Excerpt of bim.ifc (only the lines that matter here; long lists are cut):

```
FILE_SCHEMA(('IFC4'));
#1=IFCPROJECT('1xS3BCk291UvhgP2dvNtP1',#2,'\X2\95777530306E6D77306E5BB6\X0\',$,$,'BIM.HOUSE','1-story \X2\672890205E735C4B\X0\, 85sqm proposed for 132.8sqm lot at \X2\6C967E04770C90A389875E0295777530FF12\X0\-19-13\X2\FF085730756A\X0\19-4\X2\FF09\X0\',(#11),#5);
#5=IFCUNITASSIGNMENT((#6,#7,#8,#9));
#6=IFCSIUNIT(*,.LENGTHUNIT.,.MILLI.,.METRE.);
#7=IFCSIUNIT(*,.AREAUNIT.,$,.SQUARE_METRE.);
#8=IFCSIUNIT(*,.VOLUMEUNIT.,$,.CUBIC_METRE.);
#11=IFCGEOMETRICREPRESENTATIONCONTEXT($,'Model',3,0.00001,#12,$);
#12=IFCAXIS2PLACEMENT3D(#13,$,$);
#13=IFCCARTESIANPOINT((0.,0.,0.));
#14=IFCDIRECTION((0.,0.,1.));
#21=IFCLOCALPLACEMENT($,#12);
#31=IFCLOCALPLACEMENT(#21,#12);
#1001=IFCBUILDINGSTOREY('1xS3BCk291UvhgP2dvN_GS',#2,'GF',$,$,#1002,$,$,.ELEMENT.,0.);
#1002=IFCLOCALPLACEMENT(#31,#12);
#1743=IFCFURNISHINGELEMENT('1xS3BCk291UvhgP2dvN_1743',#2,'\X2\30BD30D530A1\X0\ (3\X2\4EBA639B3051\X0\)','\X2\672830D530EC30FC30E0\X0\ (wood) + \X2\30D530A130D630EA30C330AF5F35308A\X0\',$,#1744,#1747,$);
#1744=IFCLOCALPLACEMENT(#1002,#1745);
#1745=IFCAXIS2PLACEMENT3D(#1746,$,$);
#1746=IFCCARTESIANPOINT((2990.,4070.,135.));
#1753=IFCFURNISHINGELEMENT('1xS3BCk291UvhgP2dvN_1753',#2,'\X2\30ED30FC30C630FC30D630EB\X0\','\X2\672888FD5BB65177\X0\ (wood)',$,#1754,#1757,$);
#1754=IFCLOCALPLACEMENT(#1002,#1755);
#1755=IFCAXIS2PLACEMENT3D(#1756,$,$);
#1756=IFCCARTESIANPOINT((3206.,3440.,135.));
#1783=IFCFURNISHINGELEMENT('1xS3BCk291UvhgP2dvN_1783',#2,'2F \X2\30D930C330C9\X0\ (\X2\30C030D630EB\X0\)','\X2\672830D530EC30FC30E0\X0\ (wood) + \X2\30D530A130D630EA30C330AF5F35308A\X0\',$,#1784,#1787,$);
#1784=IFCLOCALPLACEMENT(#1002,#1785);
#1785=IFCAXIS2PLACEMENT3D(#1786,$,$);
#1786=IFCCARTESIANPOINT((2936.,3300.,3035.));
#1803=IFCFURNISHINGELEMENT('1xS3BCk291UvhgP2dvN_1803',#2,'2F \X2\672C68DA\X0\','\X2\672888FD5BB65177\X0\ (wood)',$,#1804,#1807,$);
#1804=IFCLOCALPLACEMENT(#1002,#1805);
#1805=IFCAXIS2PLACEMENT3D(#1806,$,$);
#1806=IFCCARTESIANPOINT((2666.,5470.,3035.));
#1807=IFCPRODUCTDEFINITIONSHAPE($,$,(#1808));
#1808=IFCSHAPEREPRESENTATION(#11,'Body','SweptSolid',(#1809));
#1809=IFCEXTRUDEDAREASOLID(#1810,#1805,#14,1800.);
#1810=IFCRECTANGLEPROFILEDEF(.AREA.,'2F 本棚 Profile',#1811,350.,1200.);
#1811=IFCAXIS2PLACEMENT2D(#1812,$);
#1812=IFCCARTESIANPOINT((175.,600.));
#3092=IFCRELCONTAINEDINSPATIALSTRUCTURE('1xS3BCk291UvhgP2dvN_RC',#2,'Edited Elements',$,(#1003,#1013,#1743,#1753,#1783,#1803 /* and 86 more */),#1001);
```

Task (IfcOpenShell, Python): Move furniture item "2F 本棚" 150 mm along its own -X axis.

```python
import ifcopenshell
import ifcopenshell.api.geometry
import ifcopenshell.util.placement
import ifcopenshell.util.unit

model = ifcopenshell.open("bim.ifc")
unit_scale = ifcopenshell.util.unit.calculate_unit_scale(model)

item = model.by_guid("1xS3BCk291UvhgP2dvN_1803")
matrix = ifcopenshell.util.placement.get_local_placement(item.ObjectPlacement)
matrix[:3, 3] -= matrix[:3, 0] * 0.15 / unit_scale
ifcopenshell.api.geometry.edit_object_placement(model, product=item, matrix=matrix, is_si=False)

print(ifcopenshell.util.placement.get_local_placement(item.ObjectPlacement).round(3) + 0.0)

model.write("bim_v2.ifc")
```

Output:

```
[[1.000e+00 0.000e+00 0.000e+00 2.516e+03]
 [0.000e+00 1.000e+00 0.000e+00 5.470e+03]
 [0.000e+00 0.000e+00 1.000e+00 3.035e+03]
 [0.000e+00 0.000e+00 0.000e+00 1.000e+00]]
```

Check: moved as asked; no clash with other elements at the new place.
